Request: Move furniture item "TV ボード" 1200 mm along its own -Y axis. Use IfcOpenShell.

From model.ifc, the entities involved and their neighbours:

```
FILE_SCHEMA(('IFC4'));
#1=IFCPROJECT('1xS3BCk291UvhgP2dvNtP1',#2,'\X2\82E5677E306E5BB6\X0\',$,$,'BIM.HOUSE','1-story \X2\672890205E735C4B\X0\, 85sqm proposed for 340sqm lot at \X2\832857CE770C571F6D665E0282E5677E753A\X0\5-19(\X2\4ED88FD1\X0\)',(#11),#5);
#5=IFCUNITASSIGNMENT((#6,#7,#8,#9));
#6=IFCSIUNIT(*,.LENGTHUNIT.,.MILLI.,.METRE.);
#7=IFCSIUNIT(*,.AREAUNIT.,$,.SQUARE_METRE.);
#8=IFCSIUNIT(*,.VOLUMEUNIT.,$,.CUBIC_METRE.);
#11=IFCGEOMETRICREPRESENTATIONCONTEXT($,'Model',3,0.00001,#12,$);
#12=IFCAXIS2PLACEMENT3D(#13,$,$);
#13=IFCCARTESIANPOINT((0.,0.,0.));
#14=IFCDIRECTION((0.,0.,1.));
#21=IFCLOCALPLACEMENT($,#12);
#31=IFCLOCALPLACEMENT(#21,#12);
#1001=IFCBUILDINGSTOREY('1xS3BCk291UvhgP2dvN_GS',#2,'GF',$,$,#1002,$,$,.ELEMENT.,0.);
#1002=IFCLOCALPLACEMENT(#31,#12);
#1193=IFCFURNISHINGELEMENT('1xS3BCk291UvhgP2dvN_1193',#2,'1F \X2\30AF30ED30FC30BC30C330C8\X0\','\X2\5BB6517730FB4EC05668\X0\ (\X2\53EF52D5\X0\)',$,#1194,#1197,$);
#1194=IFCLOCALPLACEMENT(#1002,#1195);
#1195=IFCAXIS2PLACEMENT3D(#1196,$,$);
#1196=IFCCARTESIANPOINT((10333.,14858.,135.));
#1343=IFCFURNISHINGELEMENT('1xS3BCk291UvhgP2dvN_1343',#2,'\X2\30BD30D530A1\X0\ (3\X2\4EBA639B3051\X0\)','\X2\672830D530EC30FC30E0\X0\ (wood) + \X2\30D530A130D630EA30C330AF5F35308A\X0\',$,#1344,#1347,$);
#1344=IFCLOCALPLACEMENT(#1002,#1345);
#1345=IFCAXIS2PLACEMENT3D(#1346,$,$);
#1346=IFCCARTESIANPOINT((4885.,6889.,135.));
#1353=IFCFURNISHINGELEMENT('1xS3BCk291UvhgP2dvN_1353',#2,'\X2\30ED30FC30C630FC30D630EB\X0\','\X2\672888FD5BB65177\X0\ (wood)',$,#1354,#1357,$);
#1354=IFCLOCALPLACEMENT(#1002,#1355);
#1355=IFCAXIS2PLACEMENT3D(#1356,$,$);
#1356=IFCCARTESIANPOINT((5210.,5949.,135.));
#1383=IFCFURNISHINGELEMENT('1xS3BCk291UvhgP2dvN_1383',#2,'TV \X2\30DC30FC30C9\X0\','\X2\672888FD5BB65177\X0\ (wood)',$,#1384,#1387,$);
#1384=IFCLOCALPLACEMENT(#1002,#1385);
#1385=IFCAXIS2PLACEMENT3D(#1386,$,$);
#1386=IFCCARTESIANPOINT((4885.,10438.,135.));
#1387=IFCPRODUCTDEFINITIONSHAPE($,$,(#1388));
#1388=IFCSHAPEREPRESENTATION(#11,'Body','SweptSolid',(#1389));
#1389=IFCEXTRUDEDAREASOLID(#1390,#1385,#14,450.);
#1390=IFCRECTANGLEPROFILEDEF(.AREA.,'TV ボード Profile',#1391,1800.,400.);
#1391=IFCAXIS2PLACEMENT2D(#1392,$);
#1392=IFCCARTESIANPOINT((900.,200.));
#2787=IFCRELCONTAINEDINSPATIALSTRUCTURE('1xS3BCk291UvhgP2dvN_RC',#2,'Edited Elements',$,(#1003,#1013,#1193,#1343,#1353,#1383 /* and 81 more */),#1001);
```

```python
import ifcopenshell
import ifcopenshell.api.geometry
import ifcopenshell.util.placement
import ifcopenshell.util.unit

model = ifcopenshell.open("model.ifc")
unit_scale = ifcopenshell.util.unit.calculate_unit_scale(model)

item = model.by_guid("1xS3BCk291UvhgP2dvN_1383")
matrix = ifcopenshell.util.placement.get_local_placement(item.ObjectPlacement)
matrix[:3, 3] -= matrix[:3, 1] * 1.2 / unit_scale
ifcopenshell.api.geometry.edit_object_placement(model, product=item, matrix=matrix, is_si=False)

print(ifcopenshell.util.placement.get_local_placement(item.ObjectPlacement).round(3) + 0.0)

model.write("model_updated.ifc")
```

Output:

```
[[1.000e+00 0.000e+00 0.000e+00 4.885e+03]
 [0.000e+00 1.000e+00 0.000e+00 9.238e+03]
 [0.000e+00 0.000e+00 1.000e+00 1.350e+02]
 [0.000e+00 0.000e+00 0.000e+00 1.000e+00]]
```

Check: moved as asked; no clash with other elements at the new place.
